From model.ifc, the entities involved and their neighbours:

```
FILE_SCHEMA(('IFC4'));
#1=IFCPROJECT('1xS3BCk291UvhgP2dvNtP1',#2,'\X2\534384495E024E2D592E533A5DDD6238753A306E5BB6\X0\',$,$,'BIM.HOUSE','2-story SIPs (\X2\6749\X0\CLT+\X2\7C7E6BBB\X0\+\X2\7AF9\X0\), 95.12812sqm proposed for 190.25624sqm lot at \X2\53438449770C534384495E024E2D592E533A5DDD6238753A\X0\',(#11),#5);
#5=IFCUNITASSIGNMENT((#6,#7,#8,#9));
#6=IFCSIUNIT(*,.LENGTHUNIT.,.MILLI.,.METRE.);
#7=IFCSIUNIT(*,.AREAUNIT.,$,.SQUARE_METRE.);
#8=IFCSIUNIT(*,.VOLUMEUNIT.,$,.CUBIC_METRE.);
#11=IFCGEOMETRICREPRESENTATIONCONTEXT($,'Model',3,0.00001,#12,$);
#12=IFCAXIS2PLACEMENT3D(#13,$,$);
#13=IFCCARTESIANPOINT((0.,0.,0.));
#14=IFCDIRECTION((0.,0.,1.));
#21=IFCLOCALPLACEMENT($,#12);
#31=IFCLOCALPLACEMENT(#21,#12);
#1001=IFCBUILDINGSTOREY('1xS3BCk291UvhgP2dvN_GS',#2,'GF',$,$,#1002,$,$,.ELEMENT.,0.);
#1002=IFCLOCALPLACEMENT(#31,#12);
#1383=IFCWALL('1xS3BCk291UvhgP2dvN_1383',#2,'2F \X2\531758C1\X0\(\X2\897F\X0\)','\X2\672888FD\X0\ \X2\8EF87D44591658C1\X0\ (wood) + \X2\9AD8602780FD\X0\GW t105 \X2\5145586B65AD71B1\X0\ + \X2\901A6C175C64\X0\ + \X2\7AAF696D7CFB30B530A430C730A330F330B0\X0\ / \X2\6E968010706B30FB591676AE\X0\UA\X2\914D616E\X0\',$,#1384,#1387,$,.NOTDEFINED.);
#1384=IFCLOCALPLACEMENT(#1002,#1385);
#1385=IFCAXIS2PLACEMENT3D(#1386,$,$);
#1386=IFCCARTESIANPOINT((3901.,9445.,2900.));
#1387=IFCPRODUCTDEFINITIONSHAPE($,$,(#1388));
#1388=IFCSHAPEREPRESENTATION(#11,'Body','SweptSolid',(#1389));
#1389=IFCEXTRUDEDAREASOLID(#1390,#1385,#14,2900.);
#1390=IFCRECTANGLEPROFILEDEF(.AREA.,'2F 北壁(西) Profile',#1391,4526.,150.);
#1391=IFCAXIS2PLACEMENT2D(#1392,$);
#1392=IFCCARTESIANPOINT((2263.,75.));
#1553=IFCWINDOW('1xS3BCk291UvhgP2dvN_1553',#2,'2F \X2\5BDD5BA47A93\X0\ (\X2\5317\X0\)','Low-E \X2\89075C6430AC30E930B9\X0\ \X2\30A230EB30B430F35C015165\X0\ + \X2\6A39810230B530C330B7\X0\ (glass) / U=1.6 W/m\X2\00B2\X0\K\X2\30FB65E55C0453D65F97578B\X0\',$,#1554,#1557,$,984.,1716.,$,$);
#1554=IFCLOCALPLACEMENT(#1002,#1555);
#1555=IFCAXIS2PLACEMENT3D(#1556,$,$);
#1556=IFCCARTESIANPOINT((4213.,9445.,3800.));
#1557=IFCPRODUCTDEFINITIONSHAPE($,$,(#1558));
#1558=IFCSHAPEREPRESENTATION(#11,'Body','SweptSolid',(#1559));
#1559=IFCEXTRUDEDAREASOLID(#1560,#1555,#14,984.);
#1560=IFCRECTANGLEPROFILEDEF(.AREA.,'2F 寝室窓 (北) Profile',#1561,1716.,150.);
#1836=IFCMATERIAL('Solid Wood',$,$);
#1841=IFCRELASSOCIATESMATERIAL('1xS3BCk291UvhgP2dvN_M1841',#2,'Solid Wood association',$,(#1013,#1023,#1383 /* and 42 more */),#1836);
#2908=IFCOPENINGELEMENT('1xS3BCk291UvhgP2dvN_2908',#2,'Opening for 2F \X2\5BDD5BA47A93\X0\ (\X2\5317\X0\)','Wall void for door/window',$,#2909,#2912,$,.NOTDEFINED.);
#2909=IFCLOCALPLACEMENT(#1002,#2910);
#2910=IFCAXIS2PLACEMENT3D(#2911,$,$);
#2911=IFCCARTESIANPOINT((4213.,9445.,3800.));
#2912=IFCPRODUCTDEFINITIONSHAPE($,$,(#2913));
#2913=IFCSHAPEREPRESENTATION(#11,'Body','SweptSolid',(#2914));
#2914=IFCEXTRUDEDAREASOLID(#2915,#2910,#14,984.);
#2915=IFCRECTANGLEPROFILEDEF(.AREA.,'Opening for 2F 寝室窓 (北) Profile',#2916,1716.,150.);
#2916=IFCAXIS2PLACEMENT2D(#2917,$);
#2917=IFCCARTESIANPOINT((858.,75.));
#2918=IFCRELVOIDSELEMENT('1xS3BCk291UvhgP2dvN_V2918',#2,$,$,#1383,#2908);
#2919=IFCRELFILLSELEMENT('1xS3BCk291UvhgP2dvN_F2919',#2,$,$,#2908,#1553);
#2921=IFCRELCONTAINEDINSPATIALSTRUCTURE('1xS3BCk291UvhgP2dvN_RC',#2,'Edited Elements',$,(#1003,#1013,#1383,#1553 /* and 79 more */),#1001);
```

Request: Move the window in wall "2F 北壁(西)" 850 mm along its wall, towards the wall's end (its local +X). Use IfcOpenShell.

```python
import ifcopenshell
import ifcopenshell.api.geometry
import ifcopenshell.util.placement
import ifcopenshell.util.unit

model = ifcopenshell.open("model.ifc")
unit_scale = ifcopenshell.util.unit.calculate_unit_scale(model)

window = model.by_guid("1xS3BCk291UvhgP2dvN_1553")
opening = window.FillsVoids[0].RelatingOpeningElement
wall = opening.VoidsElements[0].RelatingBuildingElement

wall_matrix = ifcopenshell.util.placement.get_local_placement(wall.ObjectPlacement)
shift = wall_matrix[:3, 0] * 0.85 / unit_scale
before = ifcopenshell.util.placement.get_local_placement(window.ObjectPlacement)[:3, 3].copy()

# The window is not placed relative to its opening, so move both.
for product in (opening, window):
    matrix = ifcopenshell.util.placement.get_local_placement(product.ObjectPlacement)
    matrix[:3, 3] += shift
    ifcopenshell.api.geometry.edit_object_placement(model, product=product, matrix=matrix, is_si=False)

after = ifcopenshell.util.placement.get_local_placement(window.ObjectPlacement)[:3, 3]
print("window moved by", (after - before).round(3) + 0.0)

model.write("model_v2.ifc")
```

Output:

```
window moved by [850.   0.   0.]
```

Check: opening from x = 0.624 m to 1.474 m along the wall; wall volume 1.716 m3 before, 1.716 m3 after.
